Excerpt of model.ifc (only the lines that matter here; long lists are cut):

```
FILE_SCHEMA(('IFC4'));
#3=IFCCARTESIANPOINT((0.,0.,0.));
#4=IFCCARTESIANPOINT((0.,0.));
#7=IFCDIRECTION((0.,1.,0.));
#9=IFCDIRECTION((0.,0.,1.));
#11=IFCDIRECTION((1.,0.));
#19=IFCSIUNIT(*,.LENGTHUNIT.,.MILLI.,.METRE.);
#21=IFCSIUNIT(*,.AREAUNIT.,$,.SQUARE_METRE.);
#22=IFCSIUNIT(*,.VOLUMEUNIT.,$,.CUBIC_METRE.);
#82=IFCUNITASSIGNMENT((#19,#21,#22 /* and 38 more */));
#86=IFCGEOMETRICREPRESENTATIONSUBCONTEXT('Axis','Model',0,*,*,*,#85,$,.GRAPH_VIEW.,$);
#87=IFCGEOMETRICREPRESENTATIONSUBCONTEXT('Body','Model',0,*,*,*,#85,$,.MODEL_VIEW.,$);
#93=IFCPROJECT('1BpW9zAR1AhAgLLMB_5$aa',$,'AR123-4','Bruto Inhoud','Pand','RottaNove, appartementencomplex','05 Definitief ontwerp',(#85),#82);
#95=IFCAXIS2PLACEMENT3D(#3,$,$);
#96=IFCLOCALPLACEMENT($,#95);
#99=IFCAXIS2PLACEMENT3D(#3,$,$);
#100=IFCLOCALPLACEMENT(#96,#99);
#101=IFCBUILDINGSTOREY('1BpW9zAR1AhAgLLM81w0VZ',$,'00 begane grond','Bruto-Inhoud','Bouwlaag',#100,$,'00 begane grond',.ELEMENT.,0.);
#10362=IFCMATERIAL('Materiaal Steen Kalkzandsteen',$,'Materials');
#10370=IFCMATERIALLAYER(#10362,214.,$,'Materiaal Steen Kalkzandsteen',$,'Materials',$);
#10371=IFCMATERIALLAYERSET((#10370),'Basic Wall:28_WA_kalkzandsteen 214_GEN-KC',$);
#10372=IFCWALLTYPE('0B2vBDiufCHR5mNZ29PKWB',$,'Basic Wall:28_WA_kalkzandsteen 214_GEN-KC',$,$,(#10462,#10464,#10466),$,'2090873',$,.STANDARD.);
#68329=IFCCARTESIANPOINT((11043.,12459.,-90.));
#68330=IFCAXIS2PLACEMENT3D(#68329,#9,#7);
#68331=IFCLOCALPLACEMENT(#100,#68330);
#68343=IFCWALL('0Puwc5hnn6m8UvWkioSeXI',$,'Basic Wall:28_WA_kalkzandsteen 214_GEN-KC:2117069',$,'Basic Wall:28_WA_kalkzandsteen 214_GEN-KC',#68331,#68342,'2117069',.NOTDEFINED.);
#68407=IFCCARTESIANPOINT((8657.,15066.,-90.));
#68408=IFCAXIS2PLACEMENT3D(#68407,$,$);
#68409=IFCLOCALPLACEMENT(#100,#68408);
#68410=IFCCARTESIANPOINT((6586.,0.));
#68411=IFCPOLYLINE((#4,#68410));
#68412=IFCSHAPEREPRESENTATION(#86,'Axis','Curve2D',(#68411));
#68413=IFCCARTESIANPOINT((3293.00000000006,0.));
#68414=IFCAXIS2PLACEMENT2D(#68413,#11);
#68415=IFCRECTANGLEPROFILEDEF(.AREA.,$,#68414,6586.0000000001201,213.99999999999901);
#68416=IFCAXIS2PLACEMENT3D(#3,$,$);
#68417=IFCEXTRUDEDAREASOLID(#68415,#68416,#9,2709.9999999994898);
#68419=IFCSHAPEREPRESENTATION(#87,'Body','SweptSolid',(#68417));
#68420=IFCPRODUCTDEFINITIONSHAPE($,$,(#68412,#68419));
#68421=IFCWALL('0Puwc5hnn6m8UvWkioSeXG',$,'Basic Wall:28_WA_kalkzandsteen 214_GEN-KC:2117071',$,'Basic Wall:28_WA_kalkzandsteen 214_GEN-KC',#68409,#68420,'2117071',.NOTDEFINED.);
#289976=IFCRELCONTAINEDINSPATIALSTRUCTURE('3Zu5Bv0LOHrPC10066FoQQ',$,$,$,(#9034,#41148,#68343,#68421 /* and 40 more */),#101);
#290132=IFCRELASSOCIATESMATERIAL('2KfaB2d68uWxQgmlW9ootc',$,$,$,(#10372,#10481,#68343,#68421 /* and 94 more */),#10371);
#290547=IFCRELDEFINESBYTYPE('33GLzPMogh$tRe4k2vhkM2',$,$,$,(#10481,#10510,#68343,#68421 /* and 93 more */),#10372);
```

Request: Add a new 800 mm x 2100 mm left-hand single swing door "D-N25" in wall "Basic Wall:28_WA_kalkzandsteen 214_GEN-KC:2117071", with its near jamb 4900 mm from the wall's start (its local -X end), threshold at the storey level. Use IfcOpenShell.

```python
import numpy as np
import ifcopenshell
import ifcopenshell.api.feature
import ifcopenshell.api.geometry
import ifcopenshell.api.root
import ifcopenshell.api.spatial
import ifcopenshell.geom
import ifcopenshell.util.element
import ifcopenshell.util.placement
import ifcopenshell.util.representation
import ifcopenshell.util.shape
import ifcopenshell.util.unit

model = ifcopenshell.open("model.ifc")
unit_scale = ifcopenshell.util.unit.calculate_unit_scale(model)
settings = ifcopenshell.geom.settings()


def volume(element):
    """Net volume in cubic metres, openings subtracted."""
    shape = ifcopenshell.geom.create_shape(settings, element)
    return ifcopenshell.util.shape.get_volume(shape.geometry)


wall = model.by_guid("0Puwc5hnn6m8UvWkioSeXG")
storey = ifcopenshell.util.element.get_container(wall, ifc_class="IfcBuildingStorey")
context = ifcopenshell.util.representation.get_context(model, "Model", "Body", "MODEL_VIEW")
before = volume(wall)

width, height, from_end, sill = 0.8, 2.1, 4.9, 0.0  # metres

# The wall runs along its own X axis, and the end named is its -X end.
wall_shape = ifcopenshell.geom.create_shape(settings, wall)
x, y, z = ifcopenshell.util.shape.get_vertices(wall_shape.geometry).T
start = x.min() + from_end
face, thickness = float(y.min()), float(y.max() - y.min())
wall_matrix = ifcopenshell.util.placement.get_local_placement(wall.ObjectPlacement)
level = ifcopenshell.util.placement.get_local_placement(storey.ObjectPlacement)[2, 3]


def in_wall(x, y):
    """Placement at x, y metres in the wall's axes, at sill height."""
    matrix = wall_matrix.copy()
    matrix[:, 3] = wall_matrix @ np.array([x / unit_scale, y / unit_scale, 0.0, 1.0])
    matrix[2, 3] = level + sill / unit_scale
    return matrix


# Opening: a box that overshoots both wall faces by 50 mm.
opening = ifcopenshell.api.root.create_entity(model, ifc_class="IfcOpeningElement", predefined_type="OPENING")
box = ifcopenshell.api.geometry.add_wall_representation(
    model, context=context, length=width, height=height, thickness=thickness + 0.1
)
ifcopenshell.api.geometry.assign_representation(model, product=opening, representation=box)
ifcopenshell.api.geometry.edit_object_placement(model, product=opening, matrix=in_wall(start, face - 0.05), is_si=False)
ifcopenshell.api.feature.add_feature(model, feature=opening, element=wall)

door = ifcopenshell.api.root.create_entity(model, ifc_class="IfcDoor", name="D-N25", predefined_type="DOOR")
door.OverallWidth, door.OverallHeight = width / unit_scale, height / unit_scale
door.OperationType = "SINGLE_SWING_LEFT"
body = ifcopenshell.api.geometry.add_door_representation(
    model,
    context=context,
    overall_width=door.OverallWidth,
    overall_height=door.OverallHeight,
    operation_type="SINGLE_SWING_LEFT",
    lining_properties={"LiningDepth": thickness / unit_scale, "ThresholdDepth": thickness / unit_scale},
)
ifcopenshell.api.geometry.assign_representation(model, product=door, representation=body)
ifcopenshell.api.spatial.assign_container(model, products=[door], relating_structure=storey)
ifcopenshell.api.feature.add_filling(model, opening=opening, element=door)

# The lining spans the wall, so the door starts at the wall face.
ifcopenshell.api.geometry.edit_object_placement(model, product=door, matrix=in_wall(start, face), is_si=False)

after = volume(wall)

print(f"wall volume {before:.3f} -> {after:.3f} m3")

model.write("model_v2.ifc")
```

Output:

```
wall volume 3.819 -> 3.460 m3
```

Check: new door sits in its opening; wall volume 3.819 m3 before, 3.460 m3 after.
